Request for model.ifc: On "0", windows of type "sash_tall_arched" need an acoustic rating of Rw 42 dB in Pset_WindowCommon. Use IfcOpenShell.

First a look at what the model holds.

```python
import ifcopenshell
import ifcopenshell.util.element

model = ifcopenshell.open("model.ifc")
print(model.schema)
storey = next(s for s in model.by_type("IfcBuildingStorey") if s.Name == "0")
windows = [e for e in ifcopenshell.util.element.get_decomposition(storey) if e.is_a("IfcWindow")]
seen = {}
for e in windows:
    element_type = ifcopenshell.util.element.get_type(e)
    key = (element_type.Name if element_type != e and element_type else None, ifcopenshell.util.element.get_pset(e, "Pset_WindowCommon", "AcousticRating"))
    seen[key] = seen.get(key, 0) + 1
for (name, value), count in sorted(seen.items(), key=str):
    print(count, "x", name, "|", value)
```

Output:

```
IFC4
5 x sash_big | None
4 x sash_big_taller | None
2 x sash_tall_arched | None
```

```python
import ifcopenshell
import ifcopenshell.api.pset
import ifcopenshell.util.element

model = ifcopenshell.open("model.ifc")

storey = next(s for s in model.by_type("IfcBuildingStorey") if s.Name == "0")
windows = [e for e in ifcopenshell.util.element.get_decomposition(storey) if e.is_a("IfcWindow")]

count = 0
for e in windows:
    element_type = ifcopenshell.util.element.get_type(e)
    if element_type in (None, e) or element_type.Name != "sash_tall_arched":
        continue
    # add_pset returns the element's existing set when there is one.
    pset = ifcopenshell.api.pset.add_pset(model, product=e, name="Pset_WindowCommon")
    ifcopenshell.api.pset.edit_pset(model, pset=pset, properties={"AcousticRating": "Rw 42 dB"})
    count += 1

print(count, "windows updated")

model.write("model-out.ifc")
```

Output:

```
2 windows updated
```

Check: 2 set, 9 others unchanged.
